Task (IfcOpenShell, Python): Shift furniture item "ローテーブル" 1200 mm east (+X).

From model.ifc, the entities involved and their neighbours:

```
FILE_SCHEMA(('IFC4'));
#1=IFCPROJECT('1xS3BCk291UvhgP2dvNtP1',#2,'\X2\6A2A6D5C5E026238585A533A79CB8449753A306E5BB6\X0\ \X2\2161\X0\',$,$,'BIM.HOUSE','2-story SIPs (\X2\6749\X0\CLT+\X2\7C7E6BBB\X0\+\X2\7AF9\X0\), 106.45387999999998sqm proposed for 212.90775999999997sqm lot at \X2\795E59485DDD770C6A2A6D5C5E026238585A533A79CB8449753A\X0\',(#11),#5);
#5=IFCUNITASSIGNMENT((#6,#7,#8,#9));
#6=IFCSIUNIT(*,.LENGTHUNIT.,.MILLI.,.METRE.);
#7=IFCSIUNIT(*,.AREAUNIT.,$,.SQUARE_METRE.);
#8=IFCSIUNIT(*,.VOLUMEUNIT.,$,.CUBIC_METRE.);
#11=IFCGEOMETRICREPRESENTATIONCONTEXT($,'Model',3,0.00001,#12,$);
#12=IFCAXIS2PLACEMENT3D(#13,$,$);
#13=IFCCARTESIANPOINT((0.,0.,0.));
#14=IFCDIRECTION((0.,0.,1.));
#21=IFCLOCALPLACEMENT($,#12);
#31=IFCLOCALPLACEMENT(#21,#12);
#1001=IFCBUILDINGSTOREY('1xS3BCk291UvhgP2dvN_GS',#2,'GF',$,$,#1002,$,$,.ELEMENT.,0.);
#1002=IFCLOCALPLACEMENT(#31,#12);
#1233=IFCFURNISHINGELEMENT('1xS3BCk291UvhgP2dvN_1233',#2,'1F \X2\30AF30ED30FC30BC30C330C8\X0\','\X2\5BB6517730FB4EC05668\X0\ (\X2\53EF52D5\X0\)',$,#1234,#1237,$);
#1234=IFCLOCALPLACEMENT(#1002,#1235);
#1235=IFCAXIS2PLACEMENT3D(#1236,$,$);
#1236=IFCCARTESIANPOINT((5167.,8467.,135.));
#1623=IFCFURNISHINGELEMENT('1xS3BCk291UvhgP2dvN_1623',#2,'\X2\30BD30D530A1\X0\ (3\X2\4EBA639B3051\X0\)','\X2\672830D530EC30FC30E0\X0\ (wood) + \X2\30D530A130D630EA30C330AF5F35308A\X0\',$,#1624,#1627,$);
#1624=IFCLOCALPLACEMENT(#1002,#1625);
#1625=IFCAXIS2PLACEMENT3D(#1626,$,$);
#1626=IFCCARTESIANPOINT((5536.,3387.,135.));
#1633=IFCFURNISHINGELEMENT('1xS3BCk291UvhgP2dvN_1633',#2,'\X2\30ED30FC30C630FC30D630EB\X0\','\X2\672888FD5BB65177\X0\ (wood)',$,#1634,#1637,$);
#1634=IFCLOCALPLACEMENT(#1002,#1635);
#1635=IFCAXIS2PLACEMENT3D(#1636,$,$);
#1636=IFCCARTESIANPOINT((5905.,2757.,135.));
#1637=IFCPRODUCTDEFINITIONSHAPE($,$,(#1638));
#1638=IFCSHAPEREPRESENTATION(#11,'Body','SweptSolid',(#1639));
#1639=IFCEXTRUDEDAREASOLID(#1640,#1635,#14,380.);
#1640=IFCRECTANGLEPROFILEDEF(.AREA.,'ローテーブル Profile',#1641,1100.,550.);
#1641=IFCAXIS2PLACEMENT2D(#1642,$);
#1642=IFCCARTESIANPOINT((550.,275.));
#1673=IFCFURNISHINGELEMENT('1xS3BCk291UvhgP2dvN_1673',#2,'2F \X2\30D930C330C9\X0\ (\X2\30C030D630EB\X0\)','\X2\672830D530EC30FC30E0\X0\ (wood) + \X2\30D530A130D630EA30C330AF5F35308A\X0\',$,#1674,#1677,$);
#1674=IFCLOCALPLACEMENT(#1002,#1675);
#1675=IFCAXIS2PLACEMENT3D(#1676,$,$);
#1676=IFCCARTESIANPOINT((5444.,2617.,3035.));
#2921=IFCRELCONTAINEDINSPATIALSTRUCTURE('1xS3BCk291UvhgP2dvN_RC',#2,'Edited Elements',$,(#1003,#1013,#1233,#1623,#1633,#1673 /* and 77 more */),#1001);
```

```python
import ifcopenshell
import ifcopenshell.api.geometry
import ifcopenshell.util.placement

model = ifcopenshell.open("model.ifc")

item = model.by_guid("1xS3BCk291UvhgP2dvN_1633")
matrix = ifcopenshell.util.placement.get_local_placement(item.ObjectPlacement)
matrix[0, 3] += 1200.0
ifcopenshell.api.geometry.edit_object_placement(model, product=item, matrix=matrix, is_si=False)

print(ifcopenshell.util.placement.get_local_placement(item.ObjectPlacement).round(3) + 0.0)

model.write("model-out.ifc")
```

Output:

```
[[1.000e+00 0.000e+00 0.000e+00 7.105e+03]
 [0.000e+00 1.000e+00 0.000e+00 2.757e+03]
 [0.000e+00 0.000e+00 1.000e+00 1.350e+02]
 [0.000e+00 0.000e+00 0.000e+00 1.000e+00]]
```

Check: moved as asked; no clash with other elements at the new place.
